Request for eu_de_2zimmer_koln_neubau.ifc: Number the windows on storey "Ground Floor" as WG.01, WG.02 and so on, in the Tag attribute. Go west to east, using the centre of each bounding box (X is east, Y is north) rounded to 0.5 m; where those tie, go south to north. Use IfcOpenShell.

First a look at what the model holds.

```python
import ifcopenshell
import ifcopenshell.util.element
import ifcopenshell.util.placement

model = ifcopenshell.open("eu_de_2zimmer_koln_neubau.ifc")
print(model.schema)
storey = next(s for s in model.by_type("IfcBuildingStorey") if s.Name == "Ground Floor")
windows = [e for e in ifcopenshell.util.element.get_decomposition(storey) if e.is_a("IfcWindow")]
for e in sorted(windows, key=lambda e: e.id()):
    origin = ifcopenshell.util.placement.get_local_placement(e.ObjectPlacement)[:3, 3]
    print(e.id(), e.Tag, e.Name, origin.round(2) + 0.0, sep=" | ")
```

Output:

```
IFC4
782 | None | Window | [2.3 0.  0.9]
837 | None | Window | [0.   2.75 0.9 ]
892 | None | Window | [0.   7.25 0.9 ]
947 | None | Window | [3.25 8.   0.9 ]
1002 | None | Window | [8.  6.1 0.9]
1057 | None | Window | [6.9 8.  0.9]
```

```python
import ifcopenshell
import ifcopenshell.geom
import ifcopenshell.util.element
import ifcopenshell.util.shape

model = ifcopenshell.open("eu_de_2zimmer_koln_neubau.ifc")
settings = ifcopenshell.geom.settings()
settings.set("use-world-coords", True)


def centre(element):
    shape = ifcopenshell.geom.create_shape(settings, element)
    return ifcopenshell.util.shape.get_bbox_centroid(shape.geometry)


storey = next(s for s in model.by_type("IfcBuildingStorey") if s.Name == "Ground Floor")
windows = [e for e in ifcopenshell.util.element.get_decomposition(storey) if e.is_a("IfcWindow")]

# Insertion points can sit at a corner or the storey origin, so sort by the geometry (in metres).
centres = {e: centre(e) for e in windows}
windows.sort(key=lambda e: (round(centres[e][0] / 0.5), centres[e][1]))

for i, e in enumerate(windows, start=1):
    number = f"WG.{i:02d}"
    e.Tag = number
    print(e.id(), number)

model.write("eu_de_2zimmer_koln_neubau_updated.ifc")
```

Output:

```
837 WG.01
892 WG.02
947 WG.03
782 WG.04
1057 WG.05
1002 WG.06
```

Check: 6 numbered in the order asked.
